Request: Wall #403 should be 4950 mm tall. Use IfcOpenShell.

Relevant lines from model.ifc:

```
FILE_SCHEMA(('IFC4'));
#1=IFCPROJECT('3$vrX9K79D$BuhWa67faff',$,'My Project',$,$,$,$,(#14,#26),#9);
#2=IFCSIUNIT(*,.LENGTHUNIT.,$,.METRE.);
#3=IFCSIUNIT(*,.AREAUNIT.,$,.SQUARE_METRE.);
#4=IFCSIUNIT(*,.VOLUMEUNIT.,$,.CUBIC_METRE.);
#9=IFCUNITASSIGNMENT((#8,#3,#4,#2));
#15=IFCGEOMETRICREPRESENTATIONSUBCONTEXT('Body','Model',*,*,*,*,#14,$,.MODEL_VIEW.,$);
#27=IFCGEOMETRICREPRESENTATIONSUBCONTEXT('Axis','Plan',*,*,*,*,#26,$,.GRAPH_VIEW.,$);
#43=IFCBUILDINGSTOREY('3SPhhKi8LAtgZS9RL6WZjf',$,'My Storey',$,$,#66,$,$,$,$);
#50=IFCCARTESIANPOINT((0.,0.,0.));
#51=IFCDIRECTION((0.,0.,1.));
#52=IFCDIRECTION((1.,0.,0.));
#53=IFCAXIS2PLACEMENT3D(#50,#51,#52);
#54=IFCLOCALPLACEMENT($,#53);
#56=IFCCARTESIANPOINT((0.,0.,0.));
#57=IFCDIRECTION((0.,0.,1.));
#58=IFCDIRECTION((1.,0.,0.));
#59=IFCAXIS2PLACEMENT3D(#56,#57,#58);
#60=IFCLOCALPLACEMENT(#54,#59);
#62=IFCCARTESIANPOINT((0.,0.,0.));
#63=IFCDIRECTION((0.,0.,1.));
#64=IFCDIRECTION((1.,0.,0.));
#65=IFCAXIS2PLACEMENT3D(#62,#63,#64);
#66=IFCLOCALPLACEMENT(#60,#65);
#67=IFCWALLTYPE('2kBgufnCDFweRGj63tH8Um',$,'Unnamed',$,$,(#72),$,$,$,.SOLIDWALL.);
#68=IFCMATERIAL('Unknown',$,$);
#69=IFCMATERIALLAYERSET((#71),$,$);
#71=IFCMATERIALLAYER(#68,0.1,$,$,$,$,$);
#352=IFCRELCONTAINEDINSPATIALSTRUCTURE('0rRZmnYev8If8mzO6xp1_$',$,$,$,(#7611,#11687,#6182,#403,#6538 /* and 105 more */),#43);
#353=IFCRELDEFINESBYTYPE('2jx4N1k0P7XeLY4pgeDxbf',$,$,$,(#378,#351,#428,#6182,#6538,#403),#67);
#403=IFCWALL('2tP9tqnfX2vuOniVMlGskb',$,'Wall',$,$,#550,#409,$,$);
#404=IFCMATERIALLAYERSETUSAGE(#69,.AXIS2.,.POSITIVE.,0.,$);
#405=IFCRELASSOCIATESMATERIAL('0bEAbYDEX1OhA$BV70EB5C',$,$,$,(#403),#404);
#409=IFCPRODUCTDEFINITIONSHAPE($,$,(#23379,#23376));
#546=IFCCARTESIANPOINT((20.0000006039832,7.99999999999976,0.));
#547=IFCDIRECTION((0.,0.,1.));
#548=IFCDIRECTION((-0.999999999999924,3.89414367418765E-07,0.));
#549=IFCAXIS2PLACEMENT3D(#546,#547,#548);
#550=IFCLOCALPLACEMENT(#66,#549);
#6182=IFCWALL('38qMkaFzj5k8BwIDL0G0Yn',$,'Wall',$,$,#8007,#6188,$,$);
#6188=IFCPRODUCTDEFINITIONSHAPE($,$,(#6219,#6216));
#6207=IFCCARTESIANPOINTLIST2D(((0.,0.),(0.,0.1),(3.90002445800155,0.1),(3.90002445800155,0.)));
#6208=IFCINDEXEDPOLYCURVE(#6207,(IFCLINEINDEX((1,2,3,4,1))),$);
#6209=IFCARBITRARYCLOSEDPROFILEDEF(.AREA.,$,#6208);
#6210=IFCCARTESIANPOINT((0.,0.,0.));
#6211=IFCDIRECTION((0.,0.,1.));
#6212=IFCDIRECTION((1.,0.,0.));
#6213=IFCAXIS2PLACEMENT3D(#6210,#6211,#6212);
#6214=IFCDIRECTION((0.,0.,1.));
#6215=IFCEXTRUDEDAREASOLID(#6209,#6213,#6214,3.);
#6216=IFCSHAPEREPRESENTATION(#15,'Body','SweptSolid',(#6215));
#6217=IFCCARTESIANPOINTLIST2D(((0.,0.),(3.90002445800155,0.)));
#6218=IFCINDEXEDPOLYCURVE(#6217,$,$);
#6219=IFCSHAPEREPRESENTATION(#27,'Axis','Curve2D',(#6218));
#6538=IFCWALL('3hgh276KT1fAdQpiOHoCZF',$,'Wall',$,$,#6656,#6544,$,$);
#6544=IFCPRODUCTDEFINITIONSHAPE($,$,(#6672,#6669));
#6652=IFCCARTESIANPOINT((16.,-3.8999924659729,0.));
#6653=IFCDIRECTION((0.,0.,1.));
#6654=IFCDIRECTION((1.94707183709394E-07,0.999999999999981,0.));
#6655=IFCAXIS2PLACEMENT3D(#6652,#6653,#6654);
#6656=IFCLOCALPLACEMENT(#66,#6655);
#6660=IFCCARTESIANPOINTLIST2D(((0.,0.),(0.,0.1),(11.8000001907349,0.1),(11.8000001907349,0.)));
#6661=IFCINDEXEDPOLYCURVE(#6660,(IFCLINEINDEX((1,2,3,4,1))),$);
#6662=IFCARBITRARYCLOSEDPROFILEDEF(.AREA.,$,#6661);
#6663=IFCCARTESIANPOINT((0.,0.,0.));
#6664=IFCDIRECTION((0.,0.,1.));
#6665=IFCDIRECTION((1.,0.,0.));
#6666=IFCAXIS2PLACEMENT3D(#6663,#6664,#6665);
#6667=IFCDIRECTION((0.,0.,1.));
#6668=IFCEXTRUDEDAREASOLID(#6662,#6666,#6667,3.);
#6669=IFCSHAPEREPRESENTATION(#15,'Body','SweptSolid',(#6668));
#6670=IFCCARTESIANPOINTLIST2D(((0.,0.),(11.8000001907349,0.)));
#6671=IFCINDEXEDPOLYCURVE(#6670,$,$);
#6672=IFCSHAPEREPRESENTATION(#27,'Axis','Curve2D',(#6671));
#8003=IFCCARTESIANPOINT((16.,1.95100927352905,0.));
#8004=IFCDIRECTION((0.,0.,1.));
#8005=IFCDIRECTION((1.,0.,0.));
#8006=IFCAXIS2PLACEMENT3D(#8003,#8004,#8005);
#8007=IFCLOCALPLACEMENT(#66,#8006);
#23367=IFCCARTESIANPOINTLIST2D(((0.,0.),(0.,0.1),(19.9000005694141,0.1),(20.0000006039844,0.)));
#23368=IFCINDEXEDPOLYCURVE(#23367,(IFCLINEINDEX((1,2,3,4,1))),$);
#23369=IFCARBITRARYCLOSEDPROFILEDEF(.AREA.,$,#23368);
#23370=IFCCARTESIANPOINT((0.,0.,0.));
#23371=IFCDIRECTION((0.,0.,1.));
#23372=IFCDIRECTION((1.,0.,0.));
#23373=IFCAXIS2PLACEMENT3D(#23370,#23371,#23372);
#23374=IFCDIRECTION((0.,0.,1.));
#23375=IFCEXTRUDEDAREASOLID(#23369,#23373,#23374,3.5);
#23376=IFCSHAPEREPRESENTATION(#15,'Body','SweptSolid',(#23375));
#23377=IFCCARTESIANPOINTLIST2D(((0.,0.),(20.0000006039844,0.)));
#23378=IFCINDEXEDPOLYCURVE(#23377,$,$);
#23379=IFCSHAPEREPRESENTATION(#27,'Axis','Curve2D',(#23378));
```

```python
import ifcopenshell
import ifcopenshell.geom
import ifcopenshell.util.representation
import ifcopenshell.util.shape

model = ifcopenshell.open("model.ifc")
settings = ifcopenshell.geom.settings()


def volume(element):
    """Net volume in cubic metres, openings subtracted."""
    shape = ifcopenshell.geom.create_shape(settings, element)
    return ifcopenshell.util.shape.get_volume(shape.geometry)


wall = model.by_guid("2tP9tqnfX2vuOniVMlGskb")
before = volume(wall)

body = ifcopenshell.util.representation.get_representation(wall, "Model", "Body")
solid = body.Items[0]
old_height = solid.Depth
solid.Depth = 4.95
after = volume(wall)

print(f"height {old_height:g} -> {solid.Depth:g}, volume {before:.3f} -> {after:.3f} m3")

model.write("model_v2.ifc")
```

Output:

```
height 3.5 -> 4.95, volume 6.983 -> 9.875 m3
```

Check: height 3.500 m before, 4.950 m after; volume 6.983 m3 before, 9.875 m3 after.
